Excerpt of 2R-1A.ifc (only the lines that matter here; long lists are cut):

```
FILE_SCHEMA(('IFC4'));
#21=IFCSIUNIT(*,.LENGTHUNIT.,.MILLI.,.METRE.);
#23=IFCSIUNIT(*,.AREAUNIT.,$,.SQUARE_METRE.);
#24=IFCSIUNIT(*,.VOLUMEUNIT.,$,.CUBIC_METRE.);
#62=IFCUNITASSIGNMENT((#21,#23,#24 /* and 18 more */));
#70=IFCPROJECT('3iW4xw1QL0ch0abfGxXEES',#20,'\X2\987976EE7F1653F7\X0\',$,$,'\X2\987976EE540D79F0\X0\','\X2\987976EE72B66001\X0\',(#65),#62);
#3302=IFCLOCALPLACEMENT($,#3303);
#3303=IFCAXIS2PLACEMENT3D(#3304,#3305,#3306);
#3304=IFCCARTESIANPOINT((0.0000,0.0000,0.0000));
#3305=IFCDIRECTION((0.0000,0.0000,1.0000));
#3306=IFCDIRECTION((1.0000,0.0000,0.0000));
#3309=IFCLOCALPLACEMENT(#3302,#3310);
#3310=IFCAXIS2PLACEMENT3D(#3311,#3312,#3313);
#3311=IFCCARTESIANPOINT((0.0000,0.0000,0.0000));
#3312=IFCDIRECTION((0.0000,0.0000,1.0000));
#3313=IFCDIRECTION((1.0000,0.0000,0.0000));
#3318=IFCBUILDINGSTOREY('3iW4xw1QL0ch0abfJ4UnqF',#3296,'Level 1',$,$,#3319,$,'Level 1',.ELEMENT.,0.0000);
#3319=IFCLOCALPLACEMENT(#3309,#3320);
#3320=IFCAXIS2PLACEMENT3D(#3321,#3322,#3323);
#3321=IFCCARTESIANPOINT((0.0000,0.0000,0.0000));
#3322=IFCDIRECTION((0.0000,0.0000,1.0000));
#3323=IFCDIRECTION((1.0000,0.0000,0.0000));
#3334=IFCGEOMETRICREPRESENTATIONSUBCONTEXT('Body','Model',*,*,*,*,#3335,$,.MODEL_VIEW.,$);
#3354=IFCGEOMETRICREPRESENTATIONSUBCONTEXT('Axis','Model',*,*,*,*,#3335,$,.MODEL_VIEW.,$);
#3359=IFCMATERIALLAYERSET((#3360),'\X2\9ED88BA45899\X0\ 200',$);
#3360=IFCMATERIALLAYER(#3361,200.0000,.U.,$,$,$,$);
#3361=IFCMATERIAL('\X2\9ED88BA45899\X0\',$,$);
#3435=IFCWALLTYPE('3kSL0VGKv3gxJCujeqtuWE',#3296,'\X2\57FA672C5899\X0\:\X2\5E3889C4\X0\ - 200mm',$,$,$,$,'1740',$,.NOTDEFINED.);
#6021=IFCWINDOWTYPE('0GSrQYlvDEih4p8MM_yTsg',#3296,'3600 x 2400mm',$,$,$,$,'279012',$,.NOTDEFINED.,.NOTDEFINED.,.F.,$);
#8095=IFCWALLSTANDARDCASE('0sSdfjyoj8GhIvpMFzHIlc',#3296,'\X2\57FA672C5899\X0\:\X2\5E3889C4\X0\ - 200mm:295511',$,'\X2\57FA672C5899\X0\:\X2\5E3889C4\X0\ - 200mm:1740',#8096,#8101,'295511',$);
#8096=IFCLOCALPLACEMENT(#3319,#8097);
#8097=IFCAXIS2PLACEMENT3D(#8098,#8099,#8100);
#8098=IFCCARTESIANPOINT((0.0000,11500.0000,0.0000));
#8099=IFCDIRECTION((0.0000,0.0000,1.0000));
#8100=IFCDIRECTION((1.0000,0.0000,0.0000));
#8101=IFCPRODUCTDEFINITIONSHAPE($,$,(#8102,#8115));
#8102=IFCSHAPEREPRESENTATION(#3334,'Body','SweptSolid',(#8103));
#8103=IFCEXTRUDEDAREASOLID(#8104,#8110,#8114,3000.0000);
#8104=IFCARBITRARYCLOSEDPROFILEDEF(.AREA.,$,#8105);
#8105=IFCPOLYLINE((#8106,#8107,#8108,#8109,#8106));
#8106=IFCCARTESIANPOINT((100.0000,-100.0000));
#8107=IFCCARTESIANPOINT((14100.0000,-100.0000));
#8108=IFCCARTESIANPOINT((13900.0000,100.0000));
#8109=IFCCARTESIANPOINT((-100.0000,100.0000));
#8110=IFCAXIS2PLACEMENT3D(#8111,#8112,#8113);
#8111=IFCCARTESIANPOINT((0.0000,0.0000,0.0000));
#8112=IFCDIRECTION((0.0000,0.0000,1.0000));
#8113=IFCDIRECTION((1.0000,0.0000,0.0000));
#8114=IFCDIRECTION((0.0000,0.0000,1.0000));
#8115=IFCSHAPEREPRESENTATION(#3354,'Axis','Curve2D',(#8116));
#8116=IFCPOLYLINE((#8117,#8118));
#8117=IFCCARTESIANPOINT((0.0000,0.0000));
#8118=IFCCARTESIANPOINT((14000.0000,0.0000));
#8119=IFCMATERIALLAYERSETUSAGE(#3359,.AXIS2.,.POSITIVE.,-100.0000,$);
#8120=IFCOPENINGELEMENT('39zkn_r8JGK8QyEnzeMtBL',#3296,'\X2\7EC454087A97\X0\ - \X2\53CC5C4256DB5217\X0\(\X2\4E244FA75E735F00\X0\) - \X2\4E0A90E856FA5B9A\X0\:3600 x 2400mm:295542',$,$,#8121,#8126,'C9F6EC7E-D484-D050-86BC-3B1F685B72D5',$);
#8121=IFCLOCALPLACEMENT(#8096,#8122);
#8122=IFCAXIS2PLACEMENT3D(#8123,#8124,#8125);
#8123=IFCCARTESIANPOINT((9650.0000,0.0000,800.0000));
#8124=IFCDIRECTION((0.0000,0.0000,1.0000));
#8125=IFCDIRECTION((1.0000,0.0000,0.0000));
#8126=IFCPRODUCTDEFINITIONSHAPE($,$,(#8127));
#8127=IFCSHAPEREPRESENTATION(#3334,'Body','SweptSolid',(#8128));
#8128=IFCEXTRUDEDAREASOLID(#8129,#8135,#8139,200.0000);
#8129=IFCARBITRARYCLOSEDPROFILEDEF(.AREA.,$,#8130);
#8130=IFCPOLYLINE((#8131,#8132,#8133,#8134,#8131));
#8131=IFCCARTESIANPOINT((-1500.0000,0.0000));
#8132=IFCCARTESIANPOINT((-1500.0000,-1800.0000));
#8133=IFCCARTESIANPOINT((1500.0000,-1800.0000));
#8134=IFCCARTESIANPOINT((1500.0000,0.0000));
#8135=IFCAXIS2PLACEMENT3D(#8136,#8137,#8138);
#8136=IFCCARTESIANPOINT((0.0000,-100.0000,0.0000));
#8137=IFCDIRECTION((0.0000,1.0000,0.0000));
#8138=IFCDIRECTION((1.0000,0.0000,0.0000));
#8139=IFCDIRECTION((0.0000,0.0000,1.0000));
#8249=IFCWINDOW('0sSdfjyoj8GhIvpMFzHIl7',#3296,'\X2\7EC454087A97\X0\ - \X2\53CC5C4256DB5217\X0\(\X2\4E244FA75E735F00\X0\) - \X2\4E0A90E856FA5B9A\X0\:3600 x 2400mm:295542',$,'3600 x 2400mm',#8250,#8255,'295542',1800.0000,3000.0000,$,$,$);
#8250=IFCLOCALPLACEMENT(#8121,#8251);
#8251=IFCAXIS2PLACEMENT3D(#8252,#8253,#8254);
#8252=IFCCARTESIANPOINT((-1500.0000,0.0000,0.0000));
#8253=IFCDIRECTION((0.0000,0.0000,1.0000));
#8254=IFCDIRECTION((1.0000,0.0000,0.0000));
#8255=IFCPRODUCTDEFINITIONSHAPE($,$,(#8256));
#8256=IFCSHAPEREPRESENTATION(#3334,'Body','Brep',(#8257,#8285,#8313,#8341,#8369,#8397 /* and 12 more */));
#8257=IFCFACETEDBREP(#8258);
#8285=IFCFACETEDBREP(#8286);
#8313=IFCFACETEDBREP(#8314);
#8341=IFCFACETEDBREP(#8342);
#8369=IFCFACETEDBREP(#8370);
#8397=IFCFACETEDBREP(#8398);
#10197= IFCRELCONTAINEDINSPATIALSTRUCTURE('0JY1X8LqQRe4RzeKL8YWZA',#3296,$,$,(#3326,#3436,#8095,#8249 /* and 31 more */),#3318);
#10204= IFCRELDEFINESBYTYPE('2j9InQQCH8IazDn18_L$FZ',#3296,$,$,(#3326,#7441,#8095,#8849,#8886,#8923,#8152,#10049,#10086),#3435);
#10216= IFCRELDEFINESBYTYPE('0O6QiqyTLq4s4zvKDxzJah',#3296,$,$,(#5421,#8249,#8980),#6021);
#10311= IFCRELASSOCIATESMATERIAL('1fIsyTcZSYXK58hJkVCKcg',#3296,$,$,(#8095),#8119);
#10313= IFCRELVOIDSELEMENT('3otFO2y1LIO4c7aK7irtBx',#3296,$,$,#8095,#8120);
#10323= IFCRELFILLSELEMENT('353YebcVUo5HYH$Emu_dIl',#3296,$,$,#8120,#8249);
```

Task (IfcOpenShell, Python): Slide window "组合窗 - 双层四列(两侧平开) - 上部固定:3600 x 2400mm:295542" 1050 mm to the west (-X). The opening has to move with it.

```python
import ifcopenshell
import ifcopenshell.api.geometry
import ifcopenshell.util.placement
import ifcopenshell.util.unit

model = ifcopenshell.open("2R-1A.ifc")
unit_scale = ifcopenshell.util.unit.calculate_unit_scale(model)

window = model.by_id(8249)
opening = window.FillsVoids[0].RelatingOpeningElement
wall = opening.VoidsElements[0].RelatingBuildingElement

wall_matrix = ifcopenshell.util.placement.get_local_placement(wall.ObjectPlacement)
shift = wall_matrix[:3, 0] * -1.05 / unit_scale
before = ifcopenshell.util.placement.get_local_placement(window.ObjectPlacement)[:3, 3].copy()

# The window is placed relative to its opening, so it follows when the opening moves.
matrix = ifcopenshell.util.placement.get_local_placement(opening.ObjectPlacement)
matrix[:3, 3] += shift
ifcopenshell.api.geometry.edit_object_placement(
    model, product=opening, matrix=matrix, is_si=False, should_transform_children=True
)

after = ifcopenshell.util.placement.get_local_placement(window.ObjectPlacement)[:3, 3]
print("window moved by", (after - before).round(3) + 0.0)

model.write("2R-1A_edited.ifc")
```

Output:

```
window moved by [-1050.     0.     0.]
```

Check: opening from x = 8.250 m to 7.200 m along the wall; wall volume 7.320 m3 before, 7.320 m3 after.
